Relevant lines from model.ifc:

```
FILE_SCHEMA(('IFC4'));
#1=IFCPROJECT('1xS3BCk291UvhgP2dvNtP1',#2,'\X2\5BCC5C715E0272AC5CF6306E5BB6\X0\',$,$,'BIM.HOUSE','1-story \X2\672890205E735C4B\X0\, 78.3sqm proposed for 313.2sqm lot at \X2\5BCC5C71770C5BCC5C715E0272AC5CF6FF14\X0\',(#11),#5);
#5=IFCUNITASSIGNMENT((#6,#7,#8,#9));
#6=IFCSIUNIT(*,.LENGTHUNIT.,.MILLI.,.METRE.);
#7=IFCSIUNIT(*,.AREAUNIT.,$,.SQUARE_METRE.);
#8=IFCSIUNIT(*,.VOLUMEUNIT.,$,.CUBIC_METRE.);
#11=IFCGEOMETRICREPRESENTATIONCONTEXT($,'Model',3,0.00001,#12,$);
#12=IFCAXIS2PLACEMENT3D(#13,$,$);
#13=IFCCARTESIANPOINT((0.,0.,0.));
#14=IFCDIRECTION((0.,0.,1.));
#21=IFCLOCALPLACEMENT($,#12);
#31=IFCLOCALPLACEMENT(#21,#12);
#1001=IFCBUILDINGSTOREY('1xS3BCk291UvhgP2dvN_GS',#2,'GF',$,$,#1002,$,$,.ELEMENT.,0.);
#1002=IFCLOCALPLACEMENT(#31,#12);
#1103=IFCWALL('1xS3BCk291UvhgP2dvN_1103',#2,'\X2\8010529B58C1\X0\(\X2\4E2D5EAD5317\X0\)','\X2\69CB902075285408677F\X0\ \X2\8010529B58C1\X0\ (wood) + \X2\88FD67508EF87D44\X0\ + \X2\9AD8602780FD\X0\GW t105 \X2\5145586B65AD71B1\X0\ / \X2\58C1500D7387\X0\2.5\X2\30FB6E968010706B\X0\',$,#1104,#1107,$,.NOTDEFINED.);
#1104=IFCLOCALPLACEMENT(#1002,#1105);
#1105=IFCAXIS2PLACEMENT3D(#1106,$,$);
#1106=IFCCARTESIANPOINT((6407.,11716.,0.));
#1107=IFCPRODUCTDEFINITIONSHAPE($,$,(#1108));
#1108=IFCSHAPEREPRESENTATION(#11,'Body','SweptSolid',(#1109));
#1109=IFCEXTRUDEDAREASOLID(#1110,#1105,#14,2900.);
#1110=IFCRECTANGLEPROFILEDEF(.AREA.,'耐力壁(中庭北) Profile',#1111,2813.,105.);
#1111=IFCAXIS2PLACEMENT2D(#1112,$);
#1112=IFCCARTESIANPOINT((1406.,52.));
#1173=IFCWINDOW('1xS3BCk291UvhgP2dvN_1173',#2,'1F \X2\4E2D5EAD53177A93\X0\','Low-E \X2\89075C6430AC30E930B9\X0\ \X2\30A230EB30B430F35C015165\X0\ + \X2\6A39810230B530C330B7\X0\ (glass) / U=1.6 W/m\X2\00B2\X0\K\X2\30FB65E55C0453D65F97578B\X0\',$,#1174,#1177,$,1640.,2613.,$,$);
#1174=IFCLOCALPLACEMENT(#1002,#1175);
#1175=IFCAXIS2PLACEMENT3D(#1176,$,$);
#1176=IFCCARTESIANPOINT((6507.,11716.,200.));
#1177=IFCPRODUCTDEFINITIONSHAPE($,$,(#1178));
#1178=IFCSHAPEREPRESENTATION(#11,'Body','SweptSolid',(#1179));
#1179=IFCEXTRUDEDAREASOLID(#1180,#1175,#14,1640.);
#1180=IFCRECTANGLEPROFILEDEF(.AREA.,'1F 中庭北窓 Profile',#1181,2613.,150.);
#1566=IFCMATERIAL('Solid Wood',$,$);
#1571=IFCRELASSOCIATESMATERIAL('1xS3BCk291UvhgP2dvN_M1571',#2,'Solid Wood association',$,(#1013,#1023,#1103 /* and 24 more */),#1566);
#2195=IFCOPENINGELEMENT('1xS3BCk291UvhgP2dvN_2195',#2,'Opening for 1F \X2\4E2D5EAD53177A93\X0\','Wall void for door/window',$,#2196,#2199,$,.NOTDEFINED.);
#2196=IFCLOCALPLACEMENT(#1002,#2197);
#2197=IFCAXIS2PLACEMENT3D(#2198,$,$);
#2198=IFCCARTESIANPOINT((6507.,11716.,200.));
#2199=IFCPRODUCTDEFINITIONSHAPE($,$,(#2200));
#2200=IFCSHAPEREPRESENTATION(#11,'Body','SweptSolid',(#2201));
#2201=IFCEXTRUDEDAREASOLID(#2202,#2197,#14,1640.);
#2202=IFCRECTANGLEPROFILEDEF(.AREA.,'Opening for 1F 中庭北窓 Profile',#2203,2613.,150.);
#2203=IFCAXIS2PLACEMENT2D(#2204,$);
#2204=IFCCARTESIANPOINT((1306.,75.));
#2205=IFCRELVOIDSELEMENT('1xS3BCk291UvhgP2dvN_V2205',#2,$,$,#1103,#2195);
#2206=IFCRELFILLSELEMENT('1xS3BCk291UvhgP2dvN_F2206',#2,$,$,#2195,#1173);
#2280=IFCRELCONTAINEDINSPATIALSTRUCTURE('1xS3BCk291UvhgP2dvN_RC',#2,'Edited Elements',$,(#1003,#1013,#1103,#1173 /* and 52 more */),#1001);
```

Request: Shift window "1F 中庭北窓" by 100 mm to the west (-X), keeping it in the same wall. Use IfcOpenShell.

```python
import ifcopenshell
import ifcopenshell.api.geometry
import ifcopenshell.util.placement
import ifcopenshell.util.unit

model = ifcopenshell.open("model.ifc")
unit_scale = ifcopenshell.util.unit.calculate_unit_scale(model)

window = model.by_guid("1xS3BCk291UvhgP2dvN_1173")
opening = window.FillsVoids[0].RelatingOpeningElement
wall = opening.VoidsElements[0].RelatingBuildingElement

wall_matrix = ifcopenshell.util.placement.get_local_placement(wall.ObjectPlacement)
shift = wall_matrix[:3, 0] * -0.1 / unit_scale
before = ifcopenshell.util.placement.get_local_placement(window.ObjectPlacement)[:3, 3].copy()

# The window is not placed relative to its opening, so move both.
for product in (opening, window):
    matrix = ifcopenshell.util.placement.get_local_placement(product.ObjectPlacement)
    matrix[:3, 3] += shift
    ifcopenshell.api.geometry.edit_object_placement(model, product=product, matrix=matrix, is_si=False)

after = ifcopenshell.util.placement.get_local_placement(window.ObjectPlacement)[:3, 3]
print("window moved by", (after - before).round(3) + 0.0)

model.write("model_edited.ifc")
```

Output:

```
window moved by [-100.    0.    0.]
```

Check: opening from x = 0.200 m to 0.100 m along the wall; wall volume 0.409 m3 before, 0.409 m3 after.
